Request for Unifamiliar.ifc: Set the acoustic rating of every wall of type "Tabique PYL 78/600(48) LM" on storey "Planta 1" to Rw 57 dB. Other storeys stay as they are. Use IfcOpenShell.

First a look at what the model holds.

```python
import ifcopenshell
import ifcopenshell.util.element

model = ifcopenshell.open("Unifamiliar.ifc")
print(model.schema)
storey = next(s for s in model.by_type("IfcBuildingStorey") if s.Name == "Planta 1")
walls = [e for e in ifcopenshell.util.element.get_decomposition(storey) if e.is_a("IfcWall")]
seen = {}
for e in walls:
    element_type = ifcopenshell.util.element.get_type(e)
    key = (element_type.Name if element_type != e and element_type else None, ifcopenshell.util.element.get_pset(e, "Pset_WallCommon", "AcousticRating"))
    seen[key] = seen.get(key, 0) + 1
for (name, value), count in sorted(seen.items(), key=str):
    print(count, "x", name, "|", value)
```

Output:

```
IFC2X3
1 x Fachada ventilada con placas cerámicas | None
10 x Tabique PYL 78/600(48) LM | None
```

```python
import ifcopenshell
import ifcopenshell.api.pset
import ifcopenshell.util.element

model = ifcopenshell.open("Unifamiliar.ifc")

storey = next(s for s in model.by_type("IfcBuildingStorey") if s.Name == "Planta 1")
walls = [e for e in ifcopenshell.util.element.get_decomposition(storey) if e.is_a("IfcWall")]

count = 0
for e in walls:
    element_type = ifcopenshell.util.element.get_type(e)
    if element_type in (None, e) or element_type.Name != "Tabique PYL 78/600(48) LM":
        continue
    # add_pset returns the element's existing set when there is one.
    pset = ifcopenshell.api.pset.add_pset(model, product=e, name="Pset_WallCommon")
    ifcopenshell.api.pset.edit_pset(model, pset=pset, properties={"AcousticRating": "Rw 57 dB"})
    count += 1

print(count, "walls updated")

model.write("Unifamiliar_rev.ifc")
```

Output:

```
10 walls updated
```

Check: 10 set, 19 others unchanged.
